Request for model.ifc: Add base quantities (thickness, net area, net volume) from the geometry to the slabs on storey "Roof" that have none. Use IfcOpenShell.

First a look at what the model holds.

```python
import ifcopenshell
import ifcopenshell.util.element
import ifcopenshell.util.unit

model = ifcopenshell.open("model.ifc")
print(model.schema)
for unit_type in ("LENGTHUNIT", "AREAUNIT", "VOLUMEUNIT"):
    print(unit_type, ifcopenshell.util.unit.calculate_unit_scale(model, unit_type))
storey = next(s for s in model.by_type("IfcBuildingStorey") if s.Name == "Roof")
slabs = [e for e in ifcopenshell.util.element.get_decomposition(storey) if e.is_a("IfcSlab")]
for e in sorted(slabs, key=lambda e: e.id()):
    print(e.id(), e.is_a(), e.Name, list(ifcopenshell.util.element.get_psets(e, qtos_only=True)), sep=" | ")
```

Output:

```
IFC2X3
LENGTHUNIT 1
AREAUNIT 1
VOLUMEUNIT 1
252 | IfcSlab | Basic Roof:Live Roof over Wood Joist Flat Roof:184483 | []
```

```python
import ifcopenshell
import ifcopenshell.api.pset
import ifcopenshell.geom
import ifcopenshell.util.element
import ifcopenshell.util.shape
import ifcopenshell.util.unit

model = ifcopenshell.open("model.ifc")
unit_scale = ifcopenshell.util.unit.calculate_unit_scale(model)
area_scale = ifcopenshell.util.unit.calculate_unit_scale(model, "AREAUNIT")
volume_scale = ifcopenshell.util.unit.calculate_unit_scale(model, "VOLUMEUNIT")
settings = ifcopenshell.geom.settings()

storey = next(s for s in model.by_type("IfcBuildingStorey") if s.Name == "Roof")
slabs = [e for e in ifcopenshell.util.element.get_decomposition(storey) if e.is_a("IfcSlab")]

for e in sorted(slabs, key=lambda e: e.id()):
    if ifcopenshell.util.element.get_psets(e, qtos_only=True, should_inherit=False):
        continue
    # Geometry comes back in metres, in the element's own axes.
    shape = ifcopenshell.geom.create_shape(settings, e)
    values = {
        "Width": ifcopenshell.util.shape.get_z(shape.geometry) / unit_scale,
        "NetArea": ifcopenshell.util.shape.get_footprint_area(shape.geometry) / area_scale,
        "NetVolume": ifcopenshell.util.shape.get_volume(shape.geometry) / volume_scale,
    }
    qto = ifcopenshell.api.pset.add_qto(model, product=e, name="BaseQuantities")
    ifcopenshell.api.pset.edit_qto(model, qto=qto, properties=values)
    print(e.id(), {k: round(v, 3) for k, v in values.items()})

model.write("model-out.ifc")
```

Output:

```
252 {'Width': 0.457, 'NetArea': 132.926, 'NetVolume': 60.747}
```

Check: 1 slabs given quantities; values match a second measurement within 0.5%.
